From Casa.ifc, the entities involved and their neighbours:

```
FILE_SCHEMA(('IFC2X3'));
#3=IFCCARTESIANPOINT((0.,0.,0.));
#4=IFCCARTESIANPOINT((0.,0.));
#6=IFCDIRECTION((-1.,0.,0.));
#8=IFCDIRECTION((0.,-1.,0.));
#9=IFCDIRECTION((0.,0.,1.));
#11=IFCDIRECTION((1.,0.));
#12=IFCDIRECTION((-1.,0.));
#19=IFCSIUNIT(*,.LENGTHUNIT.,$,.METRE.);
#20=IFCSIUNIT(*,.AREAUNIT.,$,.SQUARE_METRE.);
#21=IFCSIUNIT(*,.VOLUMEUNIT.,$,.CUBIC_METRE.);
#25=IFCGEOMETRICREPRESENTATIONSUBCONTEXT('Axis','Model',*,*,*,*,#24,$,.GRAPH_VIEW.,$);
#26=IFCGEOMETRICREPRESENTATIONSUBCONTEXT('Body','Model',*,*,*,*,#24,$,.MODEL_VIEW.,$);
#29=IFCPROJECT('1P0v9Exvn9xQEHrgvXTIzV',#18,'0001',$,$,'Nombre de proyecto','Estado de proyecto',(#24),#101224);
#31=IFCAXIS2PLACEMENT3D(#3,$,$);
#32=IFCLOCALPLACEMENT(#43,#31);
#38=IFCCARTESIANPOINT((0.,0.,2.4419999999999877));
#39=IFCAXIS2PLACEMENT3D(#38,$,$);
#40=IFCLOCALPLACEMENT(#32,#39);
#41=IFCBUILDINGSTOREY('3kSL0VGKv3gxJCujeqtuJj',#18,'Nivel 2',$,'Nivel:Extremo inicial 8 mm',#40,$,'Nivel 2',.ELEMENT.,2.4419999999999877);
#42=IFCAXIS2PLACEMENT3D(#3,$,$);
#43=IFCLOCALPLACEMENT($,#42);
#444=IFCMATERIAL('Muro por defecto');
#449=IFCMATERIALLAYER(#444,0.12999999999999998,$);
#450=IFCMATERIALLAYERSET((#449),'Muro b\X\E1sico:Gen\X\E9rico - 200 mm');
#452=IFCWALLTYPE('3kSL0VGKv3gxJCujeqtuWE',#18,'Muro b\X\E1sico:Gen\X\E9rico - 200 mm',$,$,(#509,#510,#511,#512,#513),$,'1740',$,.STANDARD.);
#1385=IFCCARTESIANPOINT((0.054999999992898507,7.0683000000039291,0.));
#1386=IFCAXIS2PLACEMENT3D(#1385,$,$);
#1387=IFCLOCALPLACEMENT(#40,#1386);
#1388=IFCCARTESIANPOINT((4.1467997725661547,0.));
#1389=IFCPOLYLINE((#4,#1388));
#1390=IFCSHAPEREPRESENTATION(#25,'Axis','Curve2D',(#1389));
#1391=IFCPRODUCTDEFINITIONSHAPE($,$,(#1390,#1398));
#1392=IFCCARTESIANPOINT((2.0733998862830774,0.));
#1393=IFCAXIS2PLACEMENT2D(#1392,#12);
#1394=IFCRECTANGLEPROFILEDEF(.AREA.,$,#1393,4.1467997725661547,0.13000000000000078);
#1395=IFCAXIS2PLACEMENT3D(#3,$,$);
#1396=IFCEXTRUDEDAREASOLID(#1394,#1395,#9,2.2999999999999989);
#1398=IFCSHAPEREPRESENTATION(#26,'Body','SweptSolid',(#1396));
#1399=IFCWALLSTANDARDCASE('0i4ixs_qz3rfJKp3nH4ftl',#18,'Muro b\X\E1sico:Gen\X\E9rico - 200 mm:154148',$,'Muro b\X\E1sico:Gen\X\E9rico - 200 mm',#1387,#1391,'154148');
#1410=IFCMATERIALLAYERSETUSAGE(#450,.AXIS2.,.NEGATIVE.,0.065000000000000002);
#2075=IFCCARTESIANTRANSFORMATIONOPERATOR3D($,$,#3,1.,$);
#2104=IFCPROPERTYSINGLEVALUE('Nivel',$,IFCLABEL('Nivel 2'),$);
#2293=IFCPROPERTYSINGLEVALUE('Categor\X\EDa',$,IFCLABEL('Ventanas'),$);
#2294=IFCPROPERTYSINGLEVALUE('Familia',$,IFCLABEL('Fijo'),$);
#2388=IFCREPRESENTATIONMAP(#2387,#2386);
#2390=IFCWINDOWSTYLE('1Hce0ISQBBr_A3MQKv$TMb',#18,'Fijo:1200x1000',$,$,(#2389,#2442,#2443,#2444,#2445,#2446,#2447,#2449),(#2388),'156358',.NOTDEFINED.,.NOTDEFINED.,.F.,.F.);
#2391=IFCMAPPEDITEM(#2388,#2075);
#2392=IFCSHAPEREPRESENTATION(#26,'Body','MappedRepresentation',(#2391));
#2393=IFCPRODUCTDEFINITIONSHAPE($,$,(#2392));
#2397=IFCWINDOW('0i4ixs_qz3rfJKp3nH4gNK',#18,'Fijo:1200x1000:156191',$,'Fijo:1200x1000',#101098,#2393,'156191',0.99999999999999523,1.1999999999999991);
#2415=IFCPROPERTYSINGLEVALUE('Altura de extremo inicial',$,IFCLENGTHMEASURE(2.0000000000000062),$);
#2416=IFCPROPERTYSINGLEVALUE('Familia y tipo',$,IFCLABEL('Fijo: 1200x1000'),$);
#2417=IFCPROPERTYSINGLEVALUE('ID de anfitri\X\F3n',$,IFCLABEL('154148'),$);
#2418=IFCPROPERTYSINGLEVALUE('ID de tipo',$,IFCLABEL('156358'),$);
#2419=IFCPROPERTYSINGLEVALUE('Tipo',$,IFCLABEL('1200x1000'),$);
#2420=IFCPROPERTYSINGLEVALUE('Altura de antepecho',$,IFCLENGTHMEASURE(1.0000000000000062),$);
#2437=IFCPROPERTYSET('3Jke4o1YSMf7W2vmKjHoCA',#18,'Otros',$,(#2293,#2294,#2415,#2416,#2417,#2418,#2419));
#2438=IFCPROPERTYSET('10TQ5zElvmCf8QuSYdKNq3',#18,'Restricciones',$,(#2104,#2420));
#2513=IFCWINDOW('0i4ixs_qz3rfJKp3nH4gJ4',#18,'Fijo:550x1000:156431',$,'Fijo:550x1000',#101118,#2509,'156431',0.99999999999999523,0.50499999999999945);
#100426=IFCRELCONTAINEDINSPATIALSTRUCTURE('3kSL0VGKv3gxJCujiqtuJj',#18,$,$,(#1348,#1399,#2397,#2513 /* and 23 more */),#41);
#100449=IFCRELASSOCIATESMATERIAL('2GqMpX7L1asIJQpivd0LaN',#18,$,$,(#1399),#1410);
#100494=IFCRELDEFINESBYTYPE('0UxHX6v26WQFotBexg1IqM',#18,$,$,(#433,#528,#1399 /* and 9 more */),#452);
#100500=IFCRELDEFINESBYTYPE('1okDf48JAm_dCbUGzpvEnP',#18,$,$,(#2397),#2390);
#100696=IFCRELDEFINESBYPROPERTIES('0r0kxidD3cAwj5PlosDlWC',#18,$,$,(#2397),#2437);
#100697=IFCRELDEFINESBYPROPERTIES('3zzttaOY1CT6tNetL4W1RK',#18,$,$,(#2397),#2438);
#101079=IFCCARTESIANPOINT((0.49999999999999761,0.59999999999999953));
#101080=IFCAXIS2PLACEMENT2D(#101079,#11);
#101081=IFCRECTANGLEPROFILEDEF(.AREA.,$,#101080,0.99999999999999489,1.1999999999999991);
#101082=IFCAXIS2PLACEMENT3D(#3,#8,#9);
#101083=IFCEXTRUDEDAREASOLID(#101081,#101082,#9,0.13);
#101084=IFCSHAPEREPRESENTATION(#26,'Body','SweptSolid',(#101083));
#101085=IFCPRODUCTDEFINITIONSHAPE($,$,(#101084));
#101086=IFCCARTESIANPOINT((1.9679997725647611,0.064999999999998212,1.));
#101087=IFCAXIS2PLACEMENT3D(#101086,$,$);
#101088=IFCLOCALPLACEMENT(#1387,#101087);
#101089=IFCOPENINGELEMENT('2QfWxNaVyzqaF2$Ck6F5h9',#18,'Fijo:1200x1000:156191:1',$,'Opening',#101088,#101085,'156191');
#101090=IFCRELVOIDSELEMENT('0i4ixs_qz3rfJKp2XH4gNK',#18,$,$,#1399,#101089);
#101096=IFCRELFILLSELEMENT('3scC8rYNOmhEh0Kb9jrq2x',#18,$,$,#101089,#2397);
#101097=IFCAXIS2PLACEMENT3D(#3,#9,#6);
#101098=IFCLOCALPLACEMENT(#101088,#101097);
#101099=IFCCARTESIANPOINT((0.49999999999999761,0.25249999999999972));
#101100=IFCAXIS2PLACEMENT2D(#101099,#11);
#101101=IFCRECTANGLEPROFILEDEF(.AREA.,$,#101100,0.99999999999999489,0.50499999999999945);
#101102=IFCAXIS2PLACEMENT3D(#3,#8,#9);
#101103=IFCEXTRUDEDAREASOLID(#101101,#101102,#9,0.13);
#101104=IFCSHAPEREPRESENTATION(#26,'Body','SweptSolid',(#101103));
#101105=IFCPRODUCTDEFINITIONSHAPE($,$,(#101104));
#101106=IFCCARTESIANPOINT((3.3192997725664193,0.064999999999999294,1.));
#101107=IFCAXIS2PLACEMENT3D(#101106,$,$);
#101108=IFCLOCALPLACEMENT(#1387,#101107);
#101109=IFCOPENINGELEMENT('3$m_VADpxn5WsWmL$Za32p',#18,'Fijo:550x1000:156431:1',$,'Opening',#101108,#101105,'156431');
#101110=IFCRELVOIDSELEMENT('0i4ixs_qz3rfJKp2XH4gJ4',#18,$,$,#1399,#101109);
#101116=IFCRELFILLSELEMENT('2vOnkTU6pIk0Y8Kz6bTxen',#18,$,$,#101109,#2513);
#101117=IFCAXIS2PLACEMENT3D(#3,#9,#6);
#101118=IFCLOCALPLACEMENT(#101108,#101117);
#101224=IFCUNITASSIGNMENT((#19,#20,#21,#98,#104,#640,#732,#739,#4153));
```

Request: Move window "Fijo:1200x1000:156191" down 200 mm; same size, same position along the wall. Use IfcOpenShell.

```python
import numpy as np
import ifcopenshell
import ifcopenshell.api.geometry
import ifcopenshell.api.pset
import ifcopenshell.util.element
import ifcopenshell.util.placement
import ifcopenshell.util.unit

model = ifcopenshell.open("Casa.ifc")
unit_scale = ifcopenshell.util.unit.calculate_unit_scale(model)

window = model.by_guid("0i4ixs_qz3rfJKp3nH4gNK")
opening = window.FillsVoids[0].RelatingOpeningElement
dz = -0.2

shift = np.array([0.0, 0.0, dz])
# The window is placed relative to its opening, so it follows when the opening moves.
matrix = ifcopenshell.util.placement.get_local_placement(opening.ObjectPlacement)
matrix[:3, 3] += shift
ifcopenshell.api.geometry.edit_object_placement(
    model, product=opening, matrix=matrix, is_si=False, should_transform_children=True
)

# Keep the stored heights in step.
pset = model.by_id(ifcopenshell.util.element.get_pset(window, "Otros", should_inherit=False)["id"])
ifcopenshell.api.pset.edit_pset(model, pset=pset, properties={
    "Altura de extremo inicial": model.create_entity("IfcLengthMeasure", ifcopenshell.util.element.get_pset(window, "Otros", "Altura de extremo inicial") + dz),
})
pset = model.by_id(ifcopenshell.util.element.get_pset(window, "Restricciones", should_inherit=False)["id"])
ifcopenshell.api.pset.edit_pset(model, pset=pset, properties={
    "Altura de antepecho": model.create_entity("IfcLengthMeasure", ifcopenshell.util.element.get_pset(window, "Restricciones", "Altura de antepecho") + dz),
})

print(f"moved by {dz * unit_scale:+.3f} m")

model.write("Casa_v2.ifc")
```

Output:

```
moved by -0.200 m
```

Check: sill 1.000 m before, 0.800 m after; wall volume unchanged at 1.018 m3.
